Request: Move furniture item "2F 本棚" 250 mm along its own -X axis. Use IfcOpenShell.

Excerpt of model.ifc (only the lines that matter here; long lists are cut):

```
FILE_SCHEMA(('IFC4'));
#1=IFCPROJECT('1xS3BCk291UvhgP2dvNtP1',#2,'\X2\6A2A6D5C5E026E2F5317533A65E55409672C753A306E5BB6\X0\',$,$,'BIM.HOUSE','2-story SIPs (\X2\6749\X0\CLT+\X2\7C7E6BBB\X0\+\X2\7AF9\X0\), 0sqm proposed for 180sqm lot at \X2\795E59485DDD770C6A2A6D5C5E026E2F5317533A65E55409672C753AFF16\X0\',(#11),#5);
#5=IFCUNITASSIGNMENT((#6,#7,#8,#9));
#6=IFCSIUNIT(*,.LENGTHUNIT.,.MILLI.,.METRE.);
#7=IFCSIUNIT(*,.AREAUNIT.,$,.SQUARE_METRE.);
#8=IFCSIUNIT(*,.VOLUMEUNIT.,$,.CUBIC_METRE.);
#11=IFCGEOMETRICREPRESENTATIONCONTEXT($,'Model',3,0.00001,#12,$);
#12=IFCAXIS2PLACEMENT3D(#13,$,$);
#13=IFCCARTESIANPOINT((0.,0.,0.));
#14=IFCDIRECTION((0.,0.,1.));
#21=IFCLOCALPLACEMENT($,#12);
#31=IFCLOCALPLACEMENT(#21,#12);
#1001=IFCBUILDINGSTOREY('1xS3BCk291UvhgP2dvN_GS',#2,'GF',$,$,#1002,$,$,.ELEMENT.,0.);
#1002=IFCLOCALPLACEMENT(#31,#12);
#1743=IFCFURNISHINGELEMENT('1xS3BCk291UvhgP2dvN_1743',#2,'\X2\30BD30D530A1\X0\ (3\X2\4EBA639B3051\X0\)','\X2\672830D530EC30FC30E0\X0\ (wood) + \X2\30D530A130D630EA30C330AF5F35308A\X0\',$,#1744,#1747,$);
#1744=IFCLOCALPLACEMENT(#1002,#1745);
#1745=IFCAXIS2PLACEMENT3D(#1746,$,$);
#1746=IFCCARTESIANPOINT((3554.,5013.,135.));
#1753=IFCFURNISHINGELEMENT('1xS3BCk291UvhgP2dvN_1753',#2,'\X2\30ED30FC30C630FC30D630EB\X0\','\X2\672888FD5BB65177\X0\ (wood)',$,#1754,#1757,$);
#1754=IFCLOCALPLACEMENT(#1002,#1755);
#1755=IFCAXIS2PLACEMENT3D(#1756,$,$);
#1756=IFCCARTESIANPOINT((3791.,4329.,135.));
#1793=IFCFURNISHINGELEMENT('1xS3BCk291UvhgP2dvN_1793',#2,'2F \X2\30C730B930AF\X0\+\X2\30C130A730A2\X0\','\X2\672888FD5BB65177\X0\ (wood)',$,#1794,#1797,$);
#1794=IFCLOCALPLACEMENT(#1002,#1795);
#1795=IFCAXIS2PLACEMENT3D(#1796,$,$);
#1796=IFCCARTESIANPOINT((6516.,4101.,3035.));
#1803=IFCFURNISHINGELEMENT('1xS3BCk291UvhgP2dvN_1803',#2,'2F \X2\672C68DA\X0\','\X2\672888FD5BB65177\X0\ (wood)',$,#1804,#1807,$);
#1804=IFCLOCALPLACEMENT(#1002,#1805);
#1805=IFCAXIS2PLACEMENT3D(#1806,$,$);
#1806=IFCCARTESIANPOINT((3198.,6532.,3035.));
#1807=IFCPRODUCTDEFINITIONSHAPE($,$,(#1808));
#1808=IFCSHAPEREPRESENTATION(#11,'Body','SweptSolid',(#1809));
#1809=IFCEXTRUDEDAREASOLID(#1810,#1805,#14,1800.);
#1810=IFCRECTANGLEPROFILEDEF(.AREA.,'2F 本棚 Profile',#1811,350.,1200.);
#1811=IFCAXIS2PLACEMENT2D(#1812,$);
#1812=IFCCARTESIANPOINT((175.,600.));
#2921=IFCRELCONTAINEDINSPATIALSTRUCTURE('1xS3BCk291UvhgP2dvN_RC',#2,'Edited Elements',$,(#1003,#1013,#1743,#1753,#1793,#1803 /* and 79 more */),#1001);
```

```python
import ifcopenshell
import ifcopenshell.api.geometry
import ifcopenshell.util.placement
import ifcopenshell.util.unit

model = ifcopenshell.open("model.ifc")
unit_scale = ifcopenshell.util.unit.calculate_unit_scale(model)

item = model.by_guid("1xS3BCk291UvhgP2dvN_1803")
matrix = ifcopenshell.util.placement.get_local_placement(item.ObjectPlacement)
matrix[:3, 3] -= matrix[:3, 0] * 0.25 / unit_scale
ifcopenshell.api.geometry.edit_object_placement(model, product=item, matrix=matrix, is_si=False)

print(ifcopenshell.util.placement.get_local_placement(item.ObjectPlacement).round(3) + 0.0)

model.write("model_updated.ifc")
```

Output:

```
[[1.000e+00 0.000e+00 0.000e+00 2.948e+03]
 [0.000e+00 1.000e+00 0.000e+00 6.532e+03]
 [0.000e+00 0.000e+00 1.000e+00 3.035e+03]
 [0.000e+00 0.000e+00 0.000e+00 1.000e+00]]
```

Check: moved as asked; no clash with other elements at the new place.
